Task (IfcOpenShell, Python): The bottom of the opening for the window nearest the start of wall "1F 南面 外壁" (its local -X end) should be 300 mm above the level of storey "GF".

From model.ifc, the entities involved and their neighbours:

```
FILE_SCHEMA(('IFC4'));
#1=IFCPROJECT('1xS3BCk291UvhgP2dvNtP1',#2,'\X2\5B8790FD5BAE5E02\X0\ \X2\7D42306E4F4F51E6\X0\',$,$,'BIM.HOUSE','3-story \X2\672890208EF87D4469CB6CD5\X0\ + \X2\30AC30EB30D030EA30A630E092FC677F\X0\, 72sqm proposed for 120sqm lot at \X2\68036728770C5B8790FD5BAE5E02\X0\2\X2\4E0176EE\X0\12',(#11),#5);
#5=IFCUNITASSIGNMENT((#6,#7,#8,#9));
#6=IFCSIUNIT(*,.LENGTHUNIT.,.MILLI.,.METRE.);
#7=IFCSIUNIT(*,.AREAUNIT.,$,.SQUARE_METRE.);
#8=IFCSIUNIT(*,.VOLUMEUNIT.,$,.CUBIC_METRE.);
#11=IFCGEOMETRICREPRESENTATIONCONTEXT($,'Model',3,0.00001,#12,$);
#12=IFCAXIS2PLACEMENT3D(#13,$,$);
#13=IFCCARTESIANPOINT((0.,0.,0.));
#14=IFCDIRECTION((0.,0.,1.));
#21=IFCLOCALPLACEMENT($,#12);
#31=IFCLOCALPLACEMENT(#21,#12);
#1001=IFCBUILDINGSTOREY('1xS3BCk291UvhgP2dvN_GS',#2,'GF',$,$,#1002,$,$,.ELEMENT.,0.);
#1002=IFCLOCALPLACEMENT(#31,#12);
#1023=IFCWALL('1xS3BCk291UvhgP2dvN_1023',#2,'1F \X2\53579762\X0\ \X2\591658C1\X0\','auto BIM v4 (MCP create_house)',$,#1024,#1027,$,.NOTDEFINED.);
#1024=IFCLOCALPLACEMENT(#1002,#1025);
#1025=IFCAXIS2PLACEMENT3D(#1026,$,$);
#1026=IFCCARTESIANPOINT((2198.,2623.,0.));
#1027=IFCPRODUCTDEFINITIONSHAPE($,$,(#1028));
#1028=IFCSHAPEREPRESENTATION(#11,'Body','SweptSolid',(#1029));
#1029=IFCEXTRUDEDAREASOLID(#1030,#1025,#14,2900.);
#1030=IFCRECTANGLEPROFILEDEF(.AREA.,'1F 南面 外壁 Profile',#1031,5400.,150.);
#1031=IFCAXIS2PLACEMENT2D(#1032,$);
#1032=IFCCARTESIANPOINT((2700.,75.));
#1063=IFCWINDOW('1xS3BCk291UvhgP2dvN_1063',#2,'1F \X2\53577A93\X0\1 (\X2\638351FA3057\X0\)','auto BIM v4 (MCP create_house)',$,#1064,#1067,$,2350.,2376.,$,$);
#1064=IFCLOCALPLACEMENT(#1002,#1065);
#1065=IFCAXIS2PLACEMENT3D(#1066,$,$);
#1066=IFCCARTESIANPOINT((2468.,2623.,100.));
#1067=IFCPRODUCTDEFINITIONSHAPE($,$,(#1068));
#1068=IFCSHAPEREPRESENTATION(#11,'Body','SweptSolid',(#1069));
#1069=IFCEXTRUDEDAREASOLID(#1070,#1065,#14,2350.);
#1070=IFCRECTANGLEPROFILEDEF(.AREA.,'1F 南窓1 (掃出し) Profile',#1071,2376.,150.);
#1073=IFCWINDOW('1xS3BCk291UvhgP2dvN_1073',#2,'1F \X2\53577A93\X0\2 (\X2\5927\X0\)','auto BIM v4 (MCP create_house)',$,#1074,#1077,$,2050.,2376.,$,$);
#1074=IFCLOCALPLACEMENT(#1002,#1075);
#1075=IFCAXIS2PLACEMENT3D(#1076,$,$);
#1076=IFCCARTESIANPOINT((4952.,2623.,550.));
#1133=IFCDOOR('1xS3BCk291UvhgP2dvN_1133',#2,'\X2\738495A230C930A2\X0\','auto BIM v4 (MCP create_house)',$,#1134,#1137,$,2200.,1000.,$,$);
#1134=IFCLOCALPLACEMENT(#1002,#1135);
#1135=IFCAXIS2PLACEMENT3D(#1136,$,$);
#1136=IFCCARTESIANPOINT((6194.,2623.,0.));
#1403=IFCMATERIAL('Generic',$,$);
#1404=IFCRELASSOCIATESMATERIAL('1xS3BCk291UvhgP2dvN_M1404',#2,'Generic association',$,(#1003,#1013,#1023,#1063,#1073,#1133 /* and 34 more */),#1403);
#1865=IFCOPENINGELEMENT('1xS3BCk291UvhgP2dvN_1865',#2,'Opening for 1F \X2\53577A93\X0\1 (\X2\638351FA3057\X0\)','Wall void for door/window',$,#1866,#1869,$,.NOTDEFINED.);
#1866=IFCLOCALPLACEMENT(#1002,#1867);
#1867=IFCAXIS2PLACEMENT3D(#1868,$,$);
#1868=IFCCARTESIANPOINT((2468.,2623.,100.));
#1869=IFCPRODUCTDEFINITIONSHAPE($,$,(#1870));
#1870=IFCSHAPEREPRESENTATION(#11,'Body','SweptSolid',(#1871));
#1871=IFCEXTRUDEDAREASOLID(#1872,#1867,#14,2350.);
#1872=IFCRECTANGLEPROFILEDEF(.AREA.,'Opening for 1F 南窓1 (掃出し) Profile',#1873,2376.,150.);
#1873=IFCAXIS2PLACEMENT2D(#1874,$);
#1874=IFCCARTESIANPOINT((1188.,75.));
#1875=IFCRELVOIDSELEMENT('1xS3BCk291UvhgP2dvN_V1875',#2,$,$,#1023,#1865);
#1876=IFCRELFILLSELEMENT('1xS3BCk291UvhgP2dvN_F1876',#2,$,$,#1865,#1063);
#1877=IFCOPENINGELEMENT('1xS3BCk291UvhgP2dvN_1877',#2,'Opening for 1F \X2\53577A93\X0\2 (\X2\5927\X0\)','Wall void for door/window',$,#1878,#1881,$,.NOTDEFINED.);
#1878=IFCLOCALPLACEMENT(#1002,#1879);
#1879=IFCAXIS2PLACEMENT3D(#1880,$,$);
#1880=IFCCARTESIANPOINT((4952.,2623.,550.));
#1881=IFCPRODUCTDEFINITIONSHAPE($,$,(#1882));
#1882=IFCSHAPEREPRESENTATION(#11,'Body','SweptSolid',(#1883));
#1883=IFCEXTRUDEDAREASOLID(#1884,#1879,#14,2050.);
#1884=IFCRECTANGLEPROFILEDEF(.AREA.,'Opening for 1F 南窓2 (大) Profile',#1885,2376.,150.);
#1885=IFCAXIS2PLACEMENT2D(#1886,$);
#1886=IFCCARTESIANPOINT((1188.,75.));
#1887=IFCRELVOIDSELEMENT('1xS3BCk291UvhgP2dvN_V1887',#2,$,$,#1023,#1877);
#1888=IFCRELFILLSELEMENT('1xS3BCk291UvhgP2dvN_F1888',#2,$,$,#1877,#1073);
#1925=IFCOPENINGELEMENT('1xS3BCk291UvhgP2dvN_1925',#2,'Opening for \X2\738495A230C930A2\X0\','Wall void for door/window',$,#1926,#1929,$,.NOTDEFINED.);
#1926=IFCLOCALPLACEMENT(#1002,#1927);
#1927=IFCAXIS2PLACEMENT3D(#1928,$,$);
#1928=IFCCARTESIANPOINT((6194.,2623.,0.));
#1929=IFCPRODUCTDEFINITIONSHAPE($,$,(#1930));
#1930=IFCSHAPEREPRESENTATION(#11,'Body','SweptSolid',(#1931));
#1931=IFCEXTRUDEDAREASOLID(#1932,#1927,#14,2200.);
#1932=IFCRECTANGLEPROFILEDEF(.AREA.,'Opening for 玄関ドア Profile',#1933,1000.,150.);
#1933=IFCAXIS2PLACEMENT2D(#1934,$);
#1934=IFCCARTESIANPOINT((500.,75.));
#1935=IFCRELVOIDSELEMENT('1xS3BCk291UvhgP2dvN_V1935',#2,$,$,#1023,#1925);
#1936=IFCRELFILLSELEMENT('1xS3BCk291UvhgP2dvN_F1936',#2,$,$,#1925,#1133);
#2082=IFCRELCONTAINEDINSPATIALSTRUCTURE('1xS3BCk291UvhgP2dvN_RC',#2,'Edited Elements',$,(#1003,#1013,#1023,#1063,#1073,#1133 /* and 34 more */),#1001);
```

```python
import numpy as np
import ifcopenshell
import ifcopenshell.api.geometry
import ifcopenshell.geom
import ifcopenshell.util.element
import ifcopenshell.util.placement
import ifcopenshell.util.shape
import ifcopenshell.util.unit

model = ifcopenshell.open("model.ifc")
unit_scale = ifcopenshell.util.unit.calculate_unit_scale(model)

window = model.by_guid("1xS3BCk291UvhgP2dvN_1063")
opening = window.FillsVoids[0].RelatingOpeningElement
storey = ifcopenshell.util.element.get_container(window, ifc_class="IfcBuildingStorey")
level = ifcopenshell.util.placement.get_local_placement(storey.ObjectPlacement)[2, 3]

# The opening's origin need not be at the sill, so measure its lowest point.
shape = ifcopenshell.geom.create_shape(ifcopenshell.geom.settings(), opening)
bottom = ifcopenshell.util.shape.get_shape_bottom_elevation(shape, shape.geometry) / unit_scale
dz = level + 300.0 - bottom

shift = np.array([0.0, 0.0, dz])
# The window is not placed relative to its opening, so move both.
for product in (opening, window):
    matrix = ifcopenshell.util.placement.get_local_placement(product.ObjectPlacement)
    matrix[:3, 3] += shift
    ifcopenshell.api.geometry.edit_object_placement(model, product=product, matrix=matrix, is_si=False)

print(f"moved by {dz * unit_scale:+.3f} m")

model.write("model_rev.ifc")
```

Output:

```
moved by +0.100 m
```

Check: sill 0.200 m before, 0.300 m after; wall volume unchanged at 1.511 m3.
